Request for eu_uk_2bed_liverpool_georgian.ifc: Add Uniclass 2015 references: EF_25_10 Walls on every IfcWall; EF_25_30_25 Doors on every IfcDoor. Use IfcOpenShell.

First a look at what the model holds.

```python
import ifcopenshell

model = ifcopenshell.open("eu_uk_2bed_liverpool_georgian.ifc")
print(model.schema)
print("classifications:", [c.Name for c in model.by_type("IfcClassification")])
for ifc_class in ("IfcDoor", "IfcRoof", "IfcStair", "IfcWall", "IfcWindow"):
    print(ifc_class, len(model.by_type(ifc_class)))
```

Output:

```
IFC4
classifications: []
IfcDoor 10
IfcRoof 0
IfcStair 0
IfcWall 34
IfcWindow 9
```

```python
import ifcopenshell
import ifcopenshell.api.classification

model = ifcopenshell.open("eu_uk_2bed_liverpool_georgian.ifc")

system = ifcopenshell.api.classification.add_classification(model, classification="Uniclass 2015")

codes = {
    "IfcWall": ("EF_25_10", "Walls"),
    "IfcDoor": ("EF_25_30_25", "Doors"),
}
for ifc_class, (code, name) in codes.items():
    products = model.by_type(ifc_class)
    ifcopenshell.api.classification.add_reference(
        model, products=products, classification=system, identification=code, name=name
    )
    print(code, len(products))

model.write("eu_uk_2bed_liverpool_georgian_v2.ifc")
```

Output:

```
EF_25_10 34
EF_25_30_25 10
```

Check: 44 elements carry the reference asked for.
